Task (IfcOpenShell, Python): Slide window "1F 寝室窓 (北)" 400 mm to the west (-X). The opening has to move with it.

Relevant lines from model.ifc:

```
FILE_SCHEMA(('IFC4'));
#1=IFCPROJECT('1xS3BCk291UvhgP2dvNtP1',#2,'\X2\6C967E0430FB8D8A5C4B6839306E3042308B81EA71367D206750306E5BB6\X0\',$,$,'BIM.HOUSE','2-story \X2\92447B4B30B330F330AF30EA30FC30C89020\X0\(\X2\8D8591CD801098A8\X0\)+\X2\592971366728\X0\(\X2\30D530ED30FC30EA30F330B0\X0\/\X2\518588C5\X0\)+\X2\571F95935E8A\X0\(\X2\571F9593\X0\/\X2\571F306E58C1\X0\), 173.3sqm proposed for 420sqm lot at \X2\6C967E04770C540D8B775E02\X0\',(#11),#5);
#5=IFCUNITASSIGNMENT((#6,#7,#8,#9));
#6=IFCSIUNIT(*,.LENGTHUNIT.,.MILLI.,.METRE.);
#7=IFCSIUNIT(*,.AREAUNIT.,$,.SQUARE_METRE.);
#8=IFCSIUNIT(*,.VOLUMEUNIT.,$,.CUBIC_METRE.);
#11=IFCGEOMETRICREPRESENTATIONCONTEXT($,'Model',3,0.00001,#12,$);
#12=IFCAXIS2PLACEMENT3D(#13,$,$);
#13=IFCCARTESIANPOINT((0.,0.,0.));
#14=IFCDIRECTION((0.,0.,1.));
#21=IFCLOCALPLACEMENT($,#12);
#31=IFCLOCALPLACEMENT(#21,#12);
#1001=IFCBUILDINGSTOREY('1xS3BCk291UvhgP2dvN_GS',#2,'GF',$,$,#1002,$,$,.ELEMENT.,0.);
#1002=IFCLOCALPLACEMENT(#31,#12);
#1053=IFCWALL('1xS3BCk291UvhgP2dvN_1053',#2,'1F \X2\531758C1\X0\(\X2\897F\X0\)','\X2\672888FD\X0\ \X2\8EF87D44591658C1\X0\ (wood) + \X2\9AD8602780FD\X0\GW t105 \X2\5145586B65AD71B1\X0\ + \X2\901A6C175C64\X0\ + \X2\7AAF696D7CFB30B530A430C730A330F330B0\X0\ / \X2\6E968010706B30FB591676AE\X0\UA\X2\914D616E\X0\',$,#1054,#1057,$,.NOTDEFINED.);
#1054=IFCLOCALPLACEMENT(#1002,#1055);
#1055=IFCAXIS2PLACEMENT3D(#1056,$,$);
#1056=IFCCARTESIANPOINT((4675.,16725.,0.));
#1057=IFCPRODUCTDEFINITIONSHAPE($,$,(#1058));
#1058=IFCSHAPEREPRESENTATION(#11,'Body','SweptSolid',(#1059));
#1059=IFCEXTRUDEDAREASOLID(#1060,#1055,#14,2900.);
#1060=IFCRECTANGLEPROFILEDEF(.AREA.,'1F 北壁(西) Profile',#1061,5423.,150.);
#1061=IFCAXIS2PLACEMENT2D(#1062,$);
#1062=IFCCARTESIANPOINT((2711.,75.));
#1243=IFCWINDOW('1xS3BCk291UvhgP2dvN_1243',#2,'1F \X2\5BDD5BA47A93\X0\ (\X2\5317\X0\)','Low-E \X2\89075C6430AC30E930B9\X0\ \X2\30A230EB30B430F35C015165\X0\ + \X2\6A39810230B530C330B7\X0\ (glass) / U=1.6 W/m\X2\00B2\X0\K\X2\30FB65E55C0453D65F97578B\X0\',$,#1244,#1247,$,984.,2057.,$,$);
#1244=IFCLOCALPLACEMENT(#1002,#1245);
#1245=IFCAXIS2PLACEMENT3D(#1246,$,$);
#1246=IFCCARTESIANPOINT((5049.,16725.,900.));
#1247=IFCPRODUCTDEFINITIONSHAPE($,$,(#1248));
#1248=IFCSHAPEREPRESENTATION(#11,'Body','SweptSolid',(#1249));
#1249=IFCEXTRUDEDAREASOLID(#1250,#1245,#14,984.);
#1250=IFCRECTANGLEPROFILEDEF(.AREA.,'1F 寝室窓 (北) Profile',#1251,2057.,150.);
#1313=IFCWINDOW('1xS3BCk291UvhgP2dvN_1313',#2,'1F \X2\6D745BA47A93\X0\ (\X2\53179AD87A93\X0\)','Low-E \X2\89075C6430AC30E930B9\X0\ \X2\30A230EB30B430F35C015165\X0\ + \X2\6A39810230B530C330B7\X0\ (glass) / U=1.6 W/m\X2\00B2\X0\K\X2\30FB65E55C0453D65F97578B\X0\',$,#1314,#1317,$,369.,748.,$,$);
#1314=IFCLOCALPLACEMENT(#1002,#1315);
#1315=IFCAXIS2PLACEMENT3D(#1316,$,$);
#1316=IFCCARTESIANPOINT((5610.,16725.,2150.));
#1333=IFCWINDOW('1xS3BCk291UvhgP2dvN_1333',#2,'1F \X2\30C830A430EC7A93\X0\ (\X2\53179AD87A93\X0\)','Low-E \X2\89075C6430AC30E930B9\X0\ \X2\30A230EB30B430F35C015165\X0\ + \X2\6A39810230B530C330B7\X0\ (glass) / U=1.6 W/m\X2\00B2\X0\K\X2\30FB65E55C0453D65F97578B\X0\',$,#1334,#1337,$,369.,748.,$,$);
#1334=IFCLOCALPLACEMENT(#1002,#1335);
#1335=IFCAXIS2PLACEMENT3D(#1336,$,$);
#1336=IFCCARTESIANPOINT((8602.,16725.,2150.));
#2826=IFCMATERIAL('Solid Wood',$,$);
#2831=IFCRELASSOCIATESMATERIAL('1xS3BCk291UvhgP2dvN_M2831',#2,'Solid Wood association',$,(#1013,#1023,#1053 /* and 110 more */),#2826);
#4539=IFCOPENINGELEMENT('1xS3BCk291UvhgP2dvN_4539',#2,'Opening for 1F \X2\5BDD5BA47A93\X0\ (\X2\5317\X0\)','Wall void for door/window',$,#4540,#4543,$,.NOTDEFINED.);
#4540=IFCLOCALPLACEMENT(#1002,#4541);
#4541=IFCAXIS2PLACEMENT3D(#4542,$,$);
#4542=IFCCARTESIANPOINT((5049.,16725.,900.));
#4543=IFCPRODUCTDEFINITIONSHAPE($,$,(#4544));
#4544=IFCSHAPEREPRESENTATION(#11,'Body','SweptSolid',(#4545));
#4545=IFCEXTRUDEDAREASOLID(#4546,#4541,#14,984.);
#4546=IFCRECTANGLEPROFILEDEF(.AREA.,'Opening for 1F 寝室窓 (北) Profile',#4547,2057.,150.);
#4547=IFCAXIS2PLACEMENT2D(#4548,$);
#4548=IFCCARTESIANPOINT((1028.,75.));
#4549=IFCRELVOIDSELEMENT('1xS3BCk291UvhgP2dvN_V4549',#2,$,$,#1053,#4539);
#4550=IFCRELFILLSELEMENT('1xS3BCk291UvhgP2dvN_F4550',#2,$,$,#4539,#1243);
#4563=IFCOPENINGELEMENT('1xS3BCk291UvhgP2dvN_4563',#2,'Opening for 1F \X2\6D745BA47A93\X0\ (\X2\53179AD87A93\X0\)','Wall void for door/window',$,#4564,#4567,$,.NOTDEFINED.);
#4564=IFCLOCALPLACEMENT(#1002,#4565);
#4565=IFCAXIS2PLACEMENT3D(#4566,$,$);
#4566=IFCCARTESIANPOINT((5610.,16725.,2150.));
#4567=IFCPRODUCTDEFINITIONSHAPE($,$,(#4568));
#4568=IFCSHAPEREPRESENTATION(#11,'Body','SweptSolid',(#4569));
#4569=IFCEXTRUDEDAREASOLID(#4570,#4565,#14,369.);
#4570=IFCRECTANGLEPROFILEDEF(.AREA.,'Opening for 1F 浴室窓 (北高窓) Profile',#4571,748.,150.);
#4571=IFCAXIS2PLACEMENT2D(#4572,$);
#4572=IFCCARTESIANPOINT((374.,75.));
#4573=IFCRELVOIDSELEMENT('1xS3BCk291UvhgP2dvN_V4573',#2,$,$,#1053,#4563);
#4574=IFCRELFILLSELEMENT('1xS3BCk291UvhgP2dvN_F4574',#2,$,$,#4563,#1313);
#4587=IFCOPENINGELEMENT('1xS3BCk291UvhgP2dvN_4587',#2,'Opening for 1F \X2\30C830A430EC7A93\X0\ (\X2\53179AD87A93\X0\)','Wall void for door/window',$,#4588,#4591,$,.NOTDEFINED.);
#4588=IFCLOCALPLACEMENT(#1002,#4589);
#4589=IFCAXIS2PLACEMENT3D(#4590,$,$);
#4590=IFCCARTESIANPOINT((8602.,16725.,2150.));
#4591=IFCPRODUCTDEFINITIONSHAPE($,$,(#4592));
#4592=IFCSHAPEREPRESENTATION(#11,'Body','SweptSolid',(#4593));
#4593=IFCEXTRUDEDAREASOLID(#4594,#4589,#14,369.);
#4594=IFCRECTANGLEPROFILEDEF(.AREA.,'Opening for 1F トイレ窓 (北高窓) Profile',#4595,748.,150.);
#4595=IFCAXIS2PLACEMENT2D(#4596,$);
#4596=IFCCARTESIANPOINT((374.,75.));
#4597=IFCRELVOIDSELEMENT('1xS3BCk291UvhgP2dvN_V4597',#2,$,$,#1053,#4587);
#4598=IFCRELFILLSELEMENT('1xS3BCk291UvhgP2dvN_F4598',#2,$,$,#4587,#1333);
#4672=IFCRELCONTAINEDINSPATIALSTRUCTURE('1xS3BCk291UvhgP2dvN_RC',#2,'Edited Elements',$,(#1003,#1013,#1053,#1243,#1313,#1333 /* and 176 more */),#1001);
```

```python
import ifcopenshell
import ifcopenshell.api.geometry
import ifcopenshell.util.placement
import ifcopenshell.util.unit

model = ifcopenshell.open("model.ifc")
unit_scale = ifcopenshell.util.unit.calculate_unit_scale(model)

window = model.by_guid("1xS3BCk291UvhgP2dvN_1243")
opening = window.FillsVoids[0].RelatingOpeningElement
wall = opening.VoidsElements[0].RelatingBuildingElement

wall_matrix = ifcopenshell.util.placement.get_local_placement(wall.ObjectPlacement)
shift = wall_matrix[:3, 0] * -0.4 / unit_scale
before = ifcopenshell.util.placement.get_local_placement(window.ObjectPlacement)[:3, 3].copy()

# The window is not placed relative to its opening, so move both.
for product in (opening, window):
    matrix = ifcopenshell.util.placement.get_local_placement(product.ObjectPlacement)
    matrix[:3, 3] += shift
    ifcopenshell.api.geometry.edit_object_placement(model, product=product, matrix=matrix, is_si=False)

after = ifcopenshell.util.placement.get_local_placement(window.ObjectPlacement)[:3, 3]
print("window moved by", (after - before).round(3) + 0.0)

model.write("model_v2.ifc")
```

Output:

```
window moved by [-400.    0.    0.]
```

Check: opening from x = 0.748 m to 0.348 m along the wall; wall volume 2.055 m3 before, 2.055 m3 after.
